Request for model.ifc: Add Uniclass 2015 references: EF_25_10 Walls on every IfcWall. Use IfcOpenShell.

First a look at what the model holds.

```python
import ifcopenshell

model = ifcopenshell.open("model.ifc")
print(model.schema)
print("classifications:", [c.Name for c in model.by_type("IfcClassification")])
for ifc_class in ("IfcDoor", "IfcRoof", "IfcStair", "IfcWall", "IfcWindow"):
    print(ifc_class, len(model.by_type(ifc_class)))
```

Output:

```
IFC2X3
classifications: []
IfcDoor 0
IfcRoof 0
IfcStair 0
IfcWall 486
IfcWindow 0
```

```python
import ifcopenshell
import ifcopenshell.api.classification

model = ifcopenshell.open("model.ifc")

# IFC2X3 requires Source and Edition and has no link from the project to the system.
system = model.create_entity("IfcClassification", Source="NBS", Edition="2015", Name="Uniclass 2015")

codes = {
    "IfcWall": ("EF_25_10", "Walls"),
}
for ifc_class, (code, name) in codes.items():
    products = model.by_type(ifc_class)
    ifcopenshell.api.classification.add_reference(
        model, products=products, classification=system, identification=code, name=name
    )
    print(code, len(products))

model.write("model-out.ifc")
```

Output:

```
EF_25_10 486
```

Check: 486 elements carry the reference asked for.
